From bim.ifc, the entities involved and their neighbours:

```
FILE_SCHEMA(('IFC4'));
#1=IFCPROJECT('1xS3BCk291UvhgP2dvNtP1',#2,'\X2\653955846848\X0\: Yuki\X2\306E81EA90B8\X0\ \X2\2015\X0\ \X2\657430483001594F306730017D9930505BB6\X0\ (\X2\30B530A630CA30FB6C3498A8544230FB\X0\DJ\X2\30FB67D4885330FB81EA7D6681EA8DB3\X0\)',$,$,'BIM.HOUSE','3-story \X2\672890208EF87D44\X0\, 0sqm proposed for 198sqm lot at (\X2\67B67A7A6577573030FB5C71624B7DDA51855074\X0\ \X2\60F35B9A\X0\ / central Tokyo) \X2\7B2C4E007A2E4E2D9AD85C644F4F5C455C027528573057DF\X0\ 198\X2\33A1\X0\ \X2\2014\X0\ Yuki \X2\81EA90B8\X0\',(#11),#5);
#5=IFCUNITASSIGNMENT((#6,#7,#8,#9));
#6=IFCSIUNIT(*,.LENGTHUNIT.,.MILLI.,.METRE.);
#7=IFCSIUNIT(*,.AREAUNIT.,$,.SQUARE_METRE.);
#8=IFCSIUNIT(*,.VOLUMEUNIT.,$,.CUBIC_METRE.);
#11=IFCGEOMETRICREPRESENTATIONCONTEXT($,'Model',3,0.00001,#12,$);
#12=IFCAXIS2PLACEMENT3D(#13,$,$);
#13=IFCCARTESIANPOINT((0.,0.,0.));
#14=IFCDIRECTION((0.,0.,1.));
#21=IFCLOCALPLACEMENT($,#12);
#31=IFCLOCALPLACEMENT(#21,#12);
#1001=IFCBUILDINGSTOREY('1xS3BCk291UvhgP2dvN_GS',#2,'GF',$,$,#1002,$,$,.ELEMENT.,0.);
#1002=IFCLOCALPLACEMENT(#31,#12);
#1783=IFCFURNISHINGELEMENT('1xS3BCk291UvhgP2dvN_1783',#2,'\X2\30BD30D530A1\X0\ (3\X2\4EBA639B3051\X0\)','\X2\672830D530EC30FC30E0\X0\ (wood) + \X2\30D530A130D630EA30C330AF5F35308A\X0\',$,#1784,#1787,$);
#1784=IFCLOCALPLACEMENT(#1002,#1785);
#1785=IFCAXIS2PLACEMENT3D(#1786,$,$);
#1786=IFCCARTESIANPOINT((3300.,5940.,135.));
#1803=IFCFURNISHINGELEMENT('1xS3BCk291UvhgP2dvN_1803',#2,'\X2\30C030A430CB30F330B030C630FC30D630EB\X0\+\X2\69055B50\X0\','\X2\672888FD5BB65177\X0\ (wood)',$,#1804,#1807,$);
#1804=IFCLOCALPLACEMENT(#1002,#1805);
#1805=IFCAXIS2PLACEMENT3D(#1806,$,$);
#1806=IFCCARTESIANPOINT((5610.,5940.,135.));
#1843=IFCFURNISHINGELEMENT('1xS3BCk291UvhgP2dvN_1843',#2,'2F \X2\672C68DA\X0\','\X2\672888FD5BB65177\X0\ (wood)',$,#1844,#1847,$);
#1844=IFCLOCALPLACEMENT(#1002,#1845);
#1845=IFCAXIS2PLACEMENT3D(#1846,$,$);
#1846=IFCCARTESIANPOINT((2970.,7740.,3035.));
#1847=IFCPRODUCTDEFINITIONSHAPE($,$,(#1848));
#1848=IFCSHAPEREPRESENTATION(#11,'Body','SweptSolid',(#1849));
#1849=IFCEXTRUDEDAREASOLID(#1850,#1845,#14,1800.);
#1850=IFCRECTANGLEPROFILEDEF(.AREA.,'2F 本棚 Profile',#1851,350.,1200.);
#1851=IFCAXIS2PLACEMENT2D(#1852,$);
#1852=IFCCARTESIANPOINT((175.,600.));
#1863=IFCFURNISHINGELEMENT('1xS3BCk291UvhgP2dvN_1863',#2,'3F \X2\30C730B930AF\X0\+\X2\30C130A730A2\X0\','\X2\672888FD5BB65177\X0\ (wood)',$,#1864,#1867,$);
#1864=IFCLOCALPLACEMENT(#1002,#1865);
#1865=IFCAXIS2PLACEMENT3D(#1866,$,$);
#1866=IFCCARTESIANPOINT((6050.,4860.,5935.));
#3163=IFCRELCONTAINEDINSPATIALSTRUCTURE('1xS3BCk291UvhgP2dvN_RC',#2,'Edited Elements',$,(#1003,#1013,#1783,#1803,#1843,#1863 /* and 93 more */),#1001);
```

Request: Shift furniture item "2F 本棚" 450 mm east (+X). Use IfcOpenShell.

```python
import ifcopenshell
import ifcopenshell.api.geometry
import ifcopenshell.util.placement

model = ifcopenshell.open("bim.ifc")

item = model.by_id(1843)
matrix = ifcopenshell.util.placement.get_local_placement(item.ObjectPlacement)
matrix[0, 3] += 450.0
ifcopenshell.api.geometry.edit_object_placement(model, product=item, matrix=matrix, is_si=False)

print(ifcopenshell.util.placement.get_local_placement(item.ObjectPlacement).round(3) + 0.0)

model.write("bim_updated.ifc")
```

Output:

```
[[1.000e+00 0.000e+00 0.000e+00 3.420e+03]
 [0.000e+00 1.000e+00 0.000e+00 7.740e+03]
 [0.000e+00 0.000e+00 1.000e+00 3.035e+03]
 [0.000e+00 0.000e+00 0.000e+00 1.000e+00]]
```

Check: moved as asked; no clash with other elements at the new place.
